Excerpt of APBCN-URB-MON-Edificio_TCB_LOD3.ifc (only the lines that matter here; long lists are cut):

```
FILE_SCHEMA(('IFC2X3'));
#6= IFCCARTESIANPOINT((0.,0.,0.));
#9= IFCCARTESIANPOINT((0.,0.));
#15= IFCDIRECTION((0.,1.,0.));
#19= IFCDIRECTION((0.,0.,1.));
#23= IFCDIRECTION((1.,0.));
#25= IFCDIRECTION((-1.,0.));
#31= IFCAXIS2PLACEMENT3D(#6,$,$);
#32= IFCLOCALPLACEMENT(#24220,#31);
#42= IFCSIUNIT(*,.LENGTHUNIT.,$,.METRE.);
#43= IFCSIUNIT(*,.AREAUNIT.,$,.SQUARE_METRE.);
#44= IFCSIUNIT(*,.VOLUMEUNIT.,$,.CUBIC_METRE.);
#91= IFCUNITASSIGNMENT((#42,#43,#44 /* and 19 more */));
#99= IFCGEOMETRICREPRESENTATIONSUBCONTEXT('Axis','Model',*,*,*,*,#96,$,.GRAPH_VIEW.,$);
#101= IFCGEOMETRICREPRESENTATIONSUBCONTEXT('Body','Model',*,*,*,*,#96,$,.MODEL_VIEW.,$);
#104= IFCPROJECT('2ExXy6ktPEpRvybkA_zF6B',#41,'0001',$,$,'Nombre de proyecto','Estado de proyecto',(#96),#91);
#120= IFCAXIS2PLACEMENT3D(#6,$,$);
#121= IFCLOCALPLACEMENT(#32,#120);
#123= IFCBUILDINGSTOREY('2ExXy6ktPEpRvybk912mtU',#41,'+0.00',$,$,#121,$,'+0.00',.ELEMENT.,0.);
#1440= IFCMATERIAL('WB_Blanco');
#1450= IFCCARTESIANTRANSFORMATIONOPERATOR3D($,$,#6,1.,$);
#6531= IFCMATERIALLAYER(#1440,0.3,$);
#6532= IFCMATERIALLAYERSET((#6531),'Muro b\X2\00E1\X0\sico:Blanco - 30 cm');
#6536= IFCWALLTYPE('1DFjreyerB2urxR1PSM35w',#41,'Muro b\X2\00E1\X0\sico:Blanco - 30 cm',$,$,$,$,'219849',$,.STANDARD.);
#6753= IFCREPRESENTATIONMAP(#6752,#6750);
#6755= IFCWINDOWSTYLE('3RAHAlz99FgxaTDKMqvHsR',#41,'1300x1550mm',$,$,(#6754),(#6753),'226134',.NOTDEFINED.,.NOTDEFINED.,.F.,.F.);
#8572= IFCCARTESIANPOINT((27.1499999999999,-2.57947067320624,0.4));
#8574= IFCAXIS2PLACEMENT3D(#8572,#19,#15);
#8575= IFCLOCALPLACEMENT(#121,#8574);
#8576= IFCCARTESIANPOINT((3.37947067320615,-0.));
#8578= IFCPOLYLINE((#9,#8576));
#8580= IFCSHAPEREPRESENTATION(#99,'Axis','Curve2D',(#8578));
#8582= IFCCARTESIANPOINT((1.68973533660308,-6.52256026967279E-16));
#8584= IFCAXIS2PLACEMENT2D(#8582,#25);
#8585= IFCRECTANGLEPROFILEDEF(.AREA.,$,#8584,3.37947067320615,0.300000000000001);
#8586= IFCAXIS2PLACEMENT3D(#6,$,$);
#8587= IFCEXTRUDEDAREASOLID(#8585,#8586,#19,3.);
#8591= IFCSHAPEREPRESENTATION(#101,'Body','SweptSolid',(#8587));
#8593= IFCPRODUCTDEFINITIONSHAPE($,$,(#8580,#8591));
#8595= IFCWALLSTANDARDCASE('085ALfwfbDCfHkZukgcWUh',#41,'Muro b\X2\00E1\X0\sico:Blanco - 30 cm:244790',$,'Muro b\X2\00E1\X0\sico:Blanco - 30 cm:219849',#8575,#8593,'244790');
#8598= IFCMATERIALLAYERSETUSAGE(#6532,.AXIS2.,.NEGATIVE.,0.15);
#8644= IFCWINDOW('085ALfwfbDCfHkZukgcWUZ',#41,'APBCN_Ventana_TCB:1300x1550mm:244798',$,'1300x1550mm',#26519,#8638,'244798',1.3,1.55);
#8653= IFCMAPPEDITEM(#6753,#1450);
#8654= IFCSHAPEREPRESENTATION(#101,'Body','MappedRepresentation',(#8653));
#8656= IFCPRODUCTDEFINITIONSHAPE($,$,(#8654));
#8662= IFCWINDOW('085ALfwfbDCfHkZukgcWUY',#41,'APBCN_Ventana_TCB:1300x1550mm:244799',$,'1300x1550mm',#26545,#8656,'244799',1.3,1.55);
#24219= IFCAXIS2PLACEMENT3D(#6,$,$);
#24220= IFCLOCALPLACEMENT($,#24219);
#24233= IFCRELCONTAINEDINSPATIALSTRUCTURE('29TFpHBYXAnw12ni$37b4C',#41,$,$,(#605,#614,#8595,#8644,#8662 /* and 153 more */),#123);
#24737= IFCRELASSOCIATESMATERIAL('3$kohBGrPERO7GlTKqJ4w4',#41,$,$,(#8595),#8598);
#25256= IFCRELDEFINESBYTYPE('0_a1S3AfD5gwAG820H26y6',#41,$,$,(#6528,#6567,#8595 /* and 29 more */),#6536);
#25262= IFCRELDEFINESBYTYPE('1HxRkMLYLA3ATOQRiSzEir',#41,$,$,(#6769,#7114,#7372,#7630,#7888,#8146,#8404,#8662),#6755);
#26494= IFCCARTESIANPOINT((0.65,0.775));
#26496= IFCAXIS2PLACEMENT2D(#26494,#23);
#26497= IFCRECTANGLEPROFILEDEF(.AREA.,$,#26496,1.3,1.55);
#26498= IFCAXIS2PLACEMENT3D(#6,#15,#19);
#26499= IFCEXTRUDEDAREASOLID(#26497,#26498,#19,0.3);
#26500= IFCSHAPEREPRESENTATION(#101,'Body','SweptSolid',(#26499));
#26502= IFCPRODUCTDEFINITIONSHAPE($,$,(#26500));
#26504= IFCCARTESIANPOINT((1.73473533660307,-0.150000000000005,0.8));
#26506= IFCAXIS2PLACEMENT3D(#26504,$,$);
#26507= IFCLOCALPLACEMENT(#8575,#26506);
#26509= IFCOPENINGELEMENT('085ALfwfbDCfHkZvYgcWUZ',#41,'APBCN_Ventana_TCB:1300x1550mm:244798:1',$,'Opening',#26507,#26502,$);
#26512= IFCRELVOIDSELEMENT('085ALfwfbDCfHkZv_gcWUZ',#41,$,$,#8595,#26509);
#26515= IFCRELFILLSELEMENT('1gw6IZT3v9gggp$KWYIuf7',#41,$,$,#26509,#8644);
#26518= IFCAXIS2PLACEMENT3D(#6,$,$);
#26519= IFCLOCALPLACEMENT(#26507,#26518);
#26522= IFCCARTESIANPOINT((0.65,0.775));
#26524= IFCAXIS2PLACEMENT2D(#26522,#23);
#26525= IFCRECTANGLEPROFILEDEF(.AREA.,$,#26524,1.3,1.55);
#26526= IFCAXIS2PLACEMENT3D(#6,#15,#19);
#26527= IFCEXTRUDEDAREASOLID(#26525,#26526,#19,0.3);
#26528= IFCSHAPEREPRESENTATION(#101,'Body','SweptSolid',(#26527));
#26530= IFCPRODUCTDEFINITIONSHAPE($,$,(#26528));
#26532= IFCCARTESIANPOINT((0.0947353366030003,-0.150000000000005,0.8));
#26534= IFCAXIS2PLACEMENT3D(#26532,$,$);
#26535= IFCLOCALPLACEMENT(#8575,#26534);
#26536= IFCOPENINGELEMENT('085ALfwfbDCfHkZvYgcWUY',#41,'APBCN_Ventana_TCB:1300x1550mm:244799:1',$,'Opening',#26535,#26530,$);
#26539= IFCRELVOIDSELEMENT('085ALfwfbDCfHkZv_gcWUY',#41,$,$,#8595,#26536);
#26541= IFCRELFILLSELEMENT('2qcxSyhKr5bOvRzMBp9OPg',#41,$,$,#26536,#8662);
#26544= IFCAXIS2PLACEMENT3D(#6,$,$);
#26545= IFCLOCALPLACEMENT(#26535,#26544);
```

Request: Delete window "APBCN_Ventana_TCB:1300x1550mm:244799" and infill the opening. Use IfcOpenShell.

```python
import ifcopenshell
import ifcopenshell.api.feature
import ifcopenshell.api.root
import ifcopenshell.geom
import ifcopenshell.util.shape

model = ifcopenshell.open("APBCN-URB-MON-Edificio_TCB_LOD3.ifc")
settings = ifcopenshell.geom.settings()


def volume(element):
    """Net volume in cubic metres, openings subtracted."""
    shape = ifcopenshell.geom.create_shape(settings, element)
    return ifcopenshell.util.shape.get_volume(shape.geometry)


window = model.by_guid("085ALfwfbDCfHkZukgcWUY")
opening = window.FillsVoids[0].RelatingOpeningElement
wall = opening.VoidsElements[0].RelatingBuildingElement
before = volume(wall)

ifcopenshell.api.root.remove_product(model, product=window)
ifcopenshell.api.feature.remove_feature(model, feature=opening)

after = volume(wall)

print(f"wall volume {before:.3f} -> {after:.3f} m3")

model.write("APBCN-URB-MON-Edificio_TCB_LOD3_v2.ifc")
```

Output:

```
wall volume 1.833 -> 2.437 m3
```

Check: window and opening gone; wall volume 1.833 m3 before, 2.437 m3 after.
